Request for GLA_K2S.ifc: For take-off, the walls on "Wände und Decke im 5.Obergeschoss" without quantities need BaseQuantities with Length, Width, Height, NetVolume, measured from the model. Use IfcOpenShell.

First a look at what the model holds.

```python
import ifcopenshell
import ifcopenshell.util.element
import ifcopenshell.util.unit

model = ifcopenshell.open("GLA_K2S.ifc")
print(model.schema)
for unit_type in ("LENGTHUNIT", "AREAUNIT", "VOLUMEUNIT"):
    print(unit_type, ifcopenshell.util.unit.calculate_unit_scale(model, unit_type))
storey = next(s for s in model.by_type("IfcBuildingStorey") if s.Name == "Wände und Decke im 5.Obergeschoss")
walls = [e for e in ifcopenshell.util.element.get_decomposition(storey) if e.is_a("IfcWall")]
for e in sorted(walls, key=lambda e: e.id()):
    print(e.id(), e.is_a(), e.Name, list(ifcopenshell.util.element.get_psets(e, qtos_only=True)), sep=" | ")
```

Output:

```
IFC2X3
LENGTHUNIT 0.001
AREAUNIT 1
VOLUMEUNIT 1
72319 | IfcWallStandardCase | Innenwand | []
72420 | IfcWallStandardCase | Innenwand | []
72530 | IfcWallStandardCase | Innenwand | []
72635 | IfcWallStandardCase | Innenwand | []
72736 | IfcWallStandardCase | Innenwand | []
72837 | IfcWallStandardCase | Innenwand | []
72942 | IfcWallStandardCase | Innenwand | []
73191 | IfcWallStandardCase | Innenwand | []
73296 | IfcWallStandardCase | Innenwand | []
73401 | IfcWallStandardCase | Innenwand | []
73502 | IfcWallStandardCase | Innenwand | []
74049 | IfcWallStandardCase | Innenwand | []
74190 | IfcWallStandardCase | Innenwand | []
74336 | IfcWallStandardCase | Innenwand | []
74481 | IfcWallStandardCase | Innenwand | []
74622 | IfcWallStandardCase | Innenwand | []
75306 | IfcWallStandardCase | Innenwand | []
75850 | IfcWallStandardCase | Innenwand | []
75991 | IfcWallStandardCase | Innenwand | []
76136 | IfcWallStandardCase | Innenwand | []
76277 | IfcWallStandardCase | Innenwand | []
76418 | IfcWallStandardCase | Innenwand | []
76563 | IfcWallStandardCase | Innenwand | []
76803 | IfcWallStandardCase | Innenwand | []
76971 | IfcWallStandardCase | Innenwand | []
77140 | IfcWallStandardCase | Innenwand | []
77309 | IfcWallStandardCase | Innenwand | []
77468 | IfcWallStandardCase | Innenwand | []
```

```python
import ifcopenshell
import ifcopenshell.api.pset
import ifcopenshell.geom
import ifcopenshell.util.element
import ifcopenshell.util.shape
import ifcopenshell.util.unit

model = ifcopenshell.open("GLA_K2S.ifc")
unit_scale = ifcopenshell.util.unit.calculate_unit_scale(model)
volume_scale = ifcopenshell.util.unit.calculate_unit_scale(model, "VOLUMEUNIT")
settings = ifcopenshell.geom.settings()

storey = next(s for s in model.by_type("IfcBuildingStorey") if s.Name == "Wände und Decke im 5.Obergeschoss")
walls = [e for e in ifcopenshell.util.element.get_decomposition(storey) if e.is_a("IfcWall")]

for e in sorted(walls, key=lambda e: e.id()):
    if ifcopenshell.util.element.get_psets(e, qtos_only=True, should_inherit=False):
        continue
    # Geometry comes back in metres, in the element's own axes.
    shape = ifcopenshell.geom.create_shape(settings, e)
    values = {
        "Length": ifcopenshell.util.shape.get_x(shape.geometry) / unit_scale,
        "Width": ifcopenshell.util.shape.get_y(shape.geometry) / unit_scale,
        "Height": ifcopenshell.util.shape.get_z(shape.geometry) / unit_scale,
        "NetVolume": ifcopenshell.util.shape.get_volume(shape.geometry) / volume_scale,
    }
    qto = ifcopenshell.api.pset.add_qto(model, product=e, name="BaseQuantities")
    ifcopenshell.api.pset.edit_qto(model, qto=qto, properties=values)
    print(e.id(), {k: round(v, 3) for k, v in values.items()})

model.write("GLA_K2S-out.ifc")
```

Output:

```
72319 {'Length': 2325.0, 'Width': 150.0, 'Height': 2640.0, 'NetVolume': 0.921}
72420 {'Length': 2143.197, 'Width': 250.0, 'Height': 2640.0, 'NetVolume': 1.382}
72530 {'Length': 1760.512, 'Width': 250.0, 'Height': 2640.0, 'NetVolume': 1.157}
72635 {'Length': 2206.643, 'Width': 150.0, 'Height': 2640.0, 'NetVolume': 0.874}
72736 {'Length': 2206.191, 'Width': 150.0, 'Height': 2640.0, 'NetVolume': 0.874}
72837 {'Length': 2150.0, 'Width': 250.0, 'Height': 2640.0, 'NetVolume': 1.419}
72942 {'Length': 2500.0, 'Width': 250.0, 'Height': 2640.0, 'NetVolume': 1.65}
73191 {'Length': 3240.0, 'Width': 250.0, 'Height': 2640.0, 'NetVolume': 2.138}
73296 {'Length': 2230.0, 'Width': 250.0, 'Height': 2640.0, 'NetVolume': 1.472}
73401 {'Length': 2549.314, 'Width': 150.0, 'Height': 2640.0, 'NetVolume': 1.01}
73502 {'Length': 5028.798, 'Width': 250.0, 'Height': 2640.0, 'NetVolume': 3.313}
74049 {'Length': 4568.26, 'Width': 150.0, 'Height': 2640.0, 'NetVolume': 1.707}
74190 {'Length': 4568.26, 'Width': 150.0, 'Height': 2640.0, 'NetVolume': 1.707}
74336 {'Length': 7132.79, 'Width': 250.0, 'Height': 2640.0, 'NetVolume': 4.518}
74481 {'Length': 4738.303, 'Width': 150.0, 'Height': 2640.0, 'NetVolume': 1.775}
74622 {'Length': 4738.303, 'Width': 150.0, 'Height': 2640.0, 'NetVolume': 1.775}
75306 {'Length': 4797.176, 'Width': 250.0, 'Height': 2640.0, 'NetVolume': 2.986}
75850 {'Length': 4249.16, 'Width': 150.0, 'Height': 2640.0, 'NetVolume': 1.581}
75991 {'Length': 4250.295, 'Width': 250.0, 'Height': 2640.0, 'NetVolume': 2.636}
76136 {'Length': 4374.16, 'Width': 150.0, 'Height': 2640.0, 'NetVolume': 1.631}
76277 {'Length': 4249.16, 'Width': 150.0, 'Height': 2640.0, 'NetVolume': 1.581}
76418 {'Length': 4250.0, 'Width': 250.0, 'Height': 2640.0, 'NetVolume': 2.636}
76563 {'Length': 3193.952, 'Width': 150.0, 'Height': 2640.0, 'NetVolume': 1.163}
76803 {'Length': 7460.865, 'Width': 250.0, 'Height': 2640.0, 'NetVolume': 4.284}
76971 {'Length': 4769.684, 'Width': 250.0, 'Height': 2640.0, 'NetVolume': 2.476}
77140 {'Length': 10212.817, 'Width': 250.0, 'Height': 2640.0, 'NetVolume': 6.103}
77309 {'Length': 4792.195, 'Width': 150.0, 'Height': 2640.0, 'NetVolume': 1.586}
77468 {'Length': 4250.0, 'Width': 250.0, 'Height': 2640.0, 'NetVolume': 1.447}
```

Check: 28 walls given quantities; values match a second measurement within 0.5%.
